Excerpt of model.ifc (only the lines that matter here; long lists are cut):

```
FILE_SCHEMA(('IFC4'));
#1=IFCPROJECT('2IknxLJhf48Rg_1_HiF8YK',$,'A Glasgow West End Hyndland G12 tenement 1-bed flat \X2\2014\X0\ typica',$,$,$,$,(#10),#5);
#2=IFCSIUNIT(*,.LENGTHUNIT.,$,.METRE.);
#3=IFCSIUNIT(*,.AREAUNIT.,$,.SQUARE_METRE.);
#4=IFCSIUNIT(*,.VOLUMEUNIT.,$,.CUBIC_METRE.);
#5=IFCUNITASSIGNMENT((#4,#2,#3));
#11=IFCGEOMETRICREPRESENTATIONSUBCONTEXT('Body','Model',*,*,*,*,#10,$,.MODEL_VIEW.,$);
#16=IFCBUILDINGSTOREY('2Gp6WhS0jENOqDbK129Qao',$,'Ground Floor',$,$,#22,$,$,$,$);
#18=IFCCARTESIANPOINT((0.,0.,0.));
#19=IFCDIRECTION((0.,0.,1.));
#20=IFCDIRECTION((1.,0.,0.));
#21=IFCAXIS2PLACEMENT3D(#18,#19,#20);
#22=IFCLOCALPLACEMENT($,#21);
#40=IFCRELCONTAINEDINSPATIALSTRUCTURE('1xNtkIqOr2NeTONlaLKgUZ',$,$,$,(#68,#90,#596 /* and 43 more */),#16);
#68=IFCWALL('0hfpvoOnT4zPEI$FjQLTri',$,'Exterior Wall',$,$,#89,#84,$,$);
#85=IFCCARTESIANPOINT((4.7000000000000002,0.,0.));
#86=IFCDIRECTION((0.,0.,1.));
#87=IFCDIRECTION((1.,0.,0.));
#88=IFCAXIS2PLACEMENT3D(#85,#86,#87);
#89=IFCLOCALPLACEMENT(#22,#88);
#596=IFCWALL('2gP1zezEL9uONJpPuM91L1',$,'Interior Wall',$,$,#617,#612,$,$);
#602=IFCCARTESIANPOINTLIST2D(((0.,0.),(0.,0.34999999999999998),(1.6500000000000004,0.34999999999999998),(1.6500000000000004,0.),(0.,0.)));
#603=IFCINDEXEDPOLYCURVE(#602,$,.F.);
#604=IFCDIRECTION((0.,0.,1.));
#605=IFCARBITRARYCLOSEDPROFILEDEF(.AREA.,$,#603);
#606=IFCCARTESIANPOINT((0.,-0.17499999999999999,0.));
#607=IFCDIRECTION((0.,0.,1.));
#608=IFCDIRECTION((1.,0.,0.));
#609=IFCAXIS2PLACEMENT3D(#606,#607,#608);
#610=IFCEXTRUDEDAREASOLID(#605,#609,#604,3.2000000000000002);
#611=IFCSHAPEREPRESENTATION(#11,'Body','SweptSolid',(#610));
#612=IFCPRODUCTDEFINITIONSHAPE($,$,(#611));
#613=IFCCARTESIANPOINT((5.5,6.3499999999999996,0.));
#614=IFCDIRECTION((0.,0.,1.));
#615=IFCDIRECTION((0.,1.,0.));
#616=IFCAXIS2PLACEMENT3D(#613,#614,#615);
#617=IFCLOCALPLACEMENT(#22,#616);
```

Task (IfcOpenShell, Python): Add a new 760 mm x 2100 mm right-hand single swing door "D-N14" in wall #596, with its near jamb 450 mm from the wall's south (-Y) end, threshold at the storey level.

```python
import numpy as np
import ifcopenshell
import ifcopenshell.api.feature
import ifcopenshell.api.geometry
import ifcopenshell.api.root
import ifcopenshell.api.spatial
import ifcopenshell.geom
import ifcopenshell.util.element
import ifcopenshell.util.placement
import ifcopenshell.util.representation
import ifcopenshell.util.shape
import ifcopenshell.util.unit

model = ifcopenshell.open("model.ifc")
unit_scale = ifcopenshell.util.unit.calculate_unit_scale(model)
settings = ifcopenshell.geom.settings()


def volume(element):
    """Net volume in cubic metres, openings subtracted."""
    shape = ifcopenshell.geom.create_shape(settings, element)
    return ifcopenshell.util.shape.get_volume(shape.geometry)


wall = model.by_id(596)
storey = ifcopenshell.util.element.get_container(wall, ifc_class="IfcBuildingStorey")
context = ifcopenshell.util.representation.get_context(model, "Model", "Body", "MODEL_VIEW")
before = volume(wall)

width, height, from_end, sill = 0.76, 2.1, 0.45, 0.0  # metres

# The wall runs along its own X axis, and the end named is its -X end.
wall_shape = ifcopenshell.geom.create_shape(settings, wall)
x, y, z = ifcopenshell.util.shape.get_vertices(wall_shape.geometry).T
start = x.min() + from_end
face, thickness = float(y.min()), float(y.max() - y.min())
wall_matrix = ifcopenshell.util.placement.get_local_placement(wall.ObjectPlacement)
level = ifcopenshell.util.placement.get_local_placement(storey.ObjectPlacement)[2, 3]


def in_wall(x, y):
    """Placement at x, y metres in the wall's axes, at sill height."""
    matrix = wall_matrix.copy()
    matrix[:, 3] = wall_matrix @ np.array([x / unit_scale, y / unit_scale, 0.0, 1.0])
    matrix[2, 3] = level + sill / unit_scale
    return matrix


# Opening: a box that overshoots both wall faces by 50 mm.
opening = ifcopenshell.api.root.create_entity(model, ifc_class="IfcOpeningElement", predefined_type="OPENING")
box = ifcopenshell.api.geometry.add_wall_representation(
    model, context=context, length=width, height=height, thickness=thickness + 0.1
)
ifcopenshell.api.geometry.assign_representation(model, product=opening, representation=box)
ifcopenshell.api.geometry.edit_object_placement(model, product=opening, matrix=in_wall(start, face - 0.05), is_si=False)
ifcopenshell.api.feature.add_feature(model, feature=opening, element=wall)

door = ifcopenshell.api.root.create_entity(model, ifc_class="IfcDoor", name="D-N14", predefined_type="DOOR")
door.OverallWidth, door.OverallHeight = width / unit_scale, height / unit_scale
door.OperationType = "SINGLE_SWING_RIGHT"
body = ifcopenshell.api.geometry.add_door_representation(
    model,
    context=context,
    overall_width=door.OverallWidth,
    overall_height=door.OverallHeight,
    operation_type="SINGLE_SWING_RIGHT",
    lining_properties={"LiningDepth": thickness / unit_scale, "ThresholdDepth": thickness / unit_scale},
)
ifcopenshell.api.geometry.assign_representation(model, product=door, representation=body)
ifcopenshell.api.spatial.assign_container(model, products=[door], relating_structure=storey)
ifcopenshell.api.feature.add_filling(model, opening=opening, element=door)

# The lining spans the wall, so the door starts at the wall face.
ifcopenshell.api.geometry.edit_object_placement(model, product=door, matrix=in_wall(start, face), is_si=False)

after = volume(wall)

print(f"wall volume {before:.3f} -> {after:.3f} m3")

model.write("model_v2.ifc")
```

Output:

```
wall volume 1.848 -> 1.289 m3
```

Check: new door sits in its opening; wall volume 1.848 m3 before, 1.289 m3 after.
